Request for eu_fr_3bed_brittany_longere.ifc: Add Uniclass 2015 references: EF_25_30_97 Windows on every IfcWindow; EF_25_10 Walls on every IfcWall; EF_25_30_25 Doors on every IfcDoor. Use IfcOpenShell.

First a look at what the model holds.

```python
import ifcopenshell

model = ifcopenshell.open("eu_fr_3bed_brittany_longere.ifc")
print(model.schema)
print("classifications:", [c.Name for c in model.by_type("IfcClassification")])
for ifc_class in ("IfcDoor", "IfcRoof", "IfcStair", "IfcWall", "IfcWindow"):
    print(ifc_class, len(model.by_type(ifc_class)))
```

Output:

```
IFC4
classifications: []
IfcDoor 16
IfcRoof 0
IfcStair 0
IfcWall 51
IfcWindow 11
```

```python
import ifcopenshell
import ifcopenshell.api.classification

model = ifcopenshell.open("eu_fr_3bed_brittany_longere.ifc")

system = ifcopenshell.api.classification.add_classification(model, classification="Uniclass 2015")

codes = {
    "IfcWindow": ("EF_25_30_97", "Windows"),
    "IfcWall": ("EF_25_10", "Walls"),
    "IfcDoor": ("EF_25_30_25", "Doors"),
}
for ifc_class, (code, name) in codes.items():
    products = model.by_type(ifc_class)
    ifcopenshell.api.classification.add_reference(
        model, products=products, classification=system, identification=code, name=name
    )
    print(code, len(products))

model.write("eu_fr_3bed_brittany_longere_edited.ifc")
```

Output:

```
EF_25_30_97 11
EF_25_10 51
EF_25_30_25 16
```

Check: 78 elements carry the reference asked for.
